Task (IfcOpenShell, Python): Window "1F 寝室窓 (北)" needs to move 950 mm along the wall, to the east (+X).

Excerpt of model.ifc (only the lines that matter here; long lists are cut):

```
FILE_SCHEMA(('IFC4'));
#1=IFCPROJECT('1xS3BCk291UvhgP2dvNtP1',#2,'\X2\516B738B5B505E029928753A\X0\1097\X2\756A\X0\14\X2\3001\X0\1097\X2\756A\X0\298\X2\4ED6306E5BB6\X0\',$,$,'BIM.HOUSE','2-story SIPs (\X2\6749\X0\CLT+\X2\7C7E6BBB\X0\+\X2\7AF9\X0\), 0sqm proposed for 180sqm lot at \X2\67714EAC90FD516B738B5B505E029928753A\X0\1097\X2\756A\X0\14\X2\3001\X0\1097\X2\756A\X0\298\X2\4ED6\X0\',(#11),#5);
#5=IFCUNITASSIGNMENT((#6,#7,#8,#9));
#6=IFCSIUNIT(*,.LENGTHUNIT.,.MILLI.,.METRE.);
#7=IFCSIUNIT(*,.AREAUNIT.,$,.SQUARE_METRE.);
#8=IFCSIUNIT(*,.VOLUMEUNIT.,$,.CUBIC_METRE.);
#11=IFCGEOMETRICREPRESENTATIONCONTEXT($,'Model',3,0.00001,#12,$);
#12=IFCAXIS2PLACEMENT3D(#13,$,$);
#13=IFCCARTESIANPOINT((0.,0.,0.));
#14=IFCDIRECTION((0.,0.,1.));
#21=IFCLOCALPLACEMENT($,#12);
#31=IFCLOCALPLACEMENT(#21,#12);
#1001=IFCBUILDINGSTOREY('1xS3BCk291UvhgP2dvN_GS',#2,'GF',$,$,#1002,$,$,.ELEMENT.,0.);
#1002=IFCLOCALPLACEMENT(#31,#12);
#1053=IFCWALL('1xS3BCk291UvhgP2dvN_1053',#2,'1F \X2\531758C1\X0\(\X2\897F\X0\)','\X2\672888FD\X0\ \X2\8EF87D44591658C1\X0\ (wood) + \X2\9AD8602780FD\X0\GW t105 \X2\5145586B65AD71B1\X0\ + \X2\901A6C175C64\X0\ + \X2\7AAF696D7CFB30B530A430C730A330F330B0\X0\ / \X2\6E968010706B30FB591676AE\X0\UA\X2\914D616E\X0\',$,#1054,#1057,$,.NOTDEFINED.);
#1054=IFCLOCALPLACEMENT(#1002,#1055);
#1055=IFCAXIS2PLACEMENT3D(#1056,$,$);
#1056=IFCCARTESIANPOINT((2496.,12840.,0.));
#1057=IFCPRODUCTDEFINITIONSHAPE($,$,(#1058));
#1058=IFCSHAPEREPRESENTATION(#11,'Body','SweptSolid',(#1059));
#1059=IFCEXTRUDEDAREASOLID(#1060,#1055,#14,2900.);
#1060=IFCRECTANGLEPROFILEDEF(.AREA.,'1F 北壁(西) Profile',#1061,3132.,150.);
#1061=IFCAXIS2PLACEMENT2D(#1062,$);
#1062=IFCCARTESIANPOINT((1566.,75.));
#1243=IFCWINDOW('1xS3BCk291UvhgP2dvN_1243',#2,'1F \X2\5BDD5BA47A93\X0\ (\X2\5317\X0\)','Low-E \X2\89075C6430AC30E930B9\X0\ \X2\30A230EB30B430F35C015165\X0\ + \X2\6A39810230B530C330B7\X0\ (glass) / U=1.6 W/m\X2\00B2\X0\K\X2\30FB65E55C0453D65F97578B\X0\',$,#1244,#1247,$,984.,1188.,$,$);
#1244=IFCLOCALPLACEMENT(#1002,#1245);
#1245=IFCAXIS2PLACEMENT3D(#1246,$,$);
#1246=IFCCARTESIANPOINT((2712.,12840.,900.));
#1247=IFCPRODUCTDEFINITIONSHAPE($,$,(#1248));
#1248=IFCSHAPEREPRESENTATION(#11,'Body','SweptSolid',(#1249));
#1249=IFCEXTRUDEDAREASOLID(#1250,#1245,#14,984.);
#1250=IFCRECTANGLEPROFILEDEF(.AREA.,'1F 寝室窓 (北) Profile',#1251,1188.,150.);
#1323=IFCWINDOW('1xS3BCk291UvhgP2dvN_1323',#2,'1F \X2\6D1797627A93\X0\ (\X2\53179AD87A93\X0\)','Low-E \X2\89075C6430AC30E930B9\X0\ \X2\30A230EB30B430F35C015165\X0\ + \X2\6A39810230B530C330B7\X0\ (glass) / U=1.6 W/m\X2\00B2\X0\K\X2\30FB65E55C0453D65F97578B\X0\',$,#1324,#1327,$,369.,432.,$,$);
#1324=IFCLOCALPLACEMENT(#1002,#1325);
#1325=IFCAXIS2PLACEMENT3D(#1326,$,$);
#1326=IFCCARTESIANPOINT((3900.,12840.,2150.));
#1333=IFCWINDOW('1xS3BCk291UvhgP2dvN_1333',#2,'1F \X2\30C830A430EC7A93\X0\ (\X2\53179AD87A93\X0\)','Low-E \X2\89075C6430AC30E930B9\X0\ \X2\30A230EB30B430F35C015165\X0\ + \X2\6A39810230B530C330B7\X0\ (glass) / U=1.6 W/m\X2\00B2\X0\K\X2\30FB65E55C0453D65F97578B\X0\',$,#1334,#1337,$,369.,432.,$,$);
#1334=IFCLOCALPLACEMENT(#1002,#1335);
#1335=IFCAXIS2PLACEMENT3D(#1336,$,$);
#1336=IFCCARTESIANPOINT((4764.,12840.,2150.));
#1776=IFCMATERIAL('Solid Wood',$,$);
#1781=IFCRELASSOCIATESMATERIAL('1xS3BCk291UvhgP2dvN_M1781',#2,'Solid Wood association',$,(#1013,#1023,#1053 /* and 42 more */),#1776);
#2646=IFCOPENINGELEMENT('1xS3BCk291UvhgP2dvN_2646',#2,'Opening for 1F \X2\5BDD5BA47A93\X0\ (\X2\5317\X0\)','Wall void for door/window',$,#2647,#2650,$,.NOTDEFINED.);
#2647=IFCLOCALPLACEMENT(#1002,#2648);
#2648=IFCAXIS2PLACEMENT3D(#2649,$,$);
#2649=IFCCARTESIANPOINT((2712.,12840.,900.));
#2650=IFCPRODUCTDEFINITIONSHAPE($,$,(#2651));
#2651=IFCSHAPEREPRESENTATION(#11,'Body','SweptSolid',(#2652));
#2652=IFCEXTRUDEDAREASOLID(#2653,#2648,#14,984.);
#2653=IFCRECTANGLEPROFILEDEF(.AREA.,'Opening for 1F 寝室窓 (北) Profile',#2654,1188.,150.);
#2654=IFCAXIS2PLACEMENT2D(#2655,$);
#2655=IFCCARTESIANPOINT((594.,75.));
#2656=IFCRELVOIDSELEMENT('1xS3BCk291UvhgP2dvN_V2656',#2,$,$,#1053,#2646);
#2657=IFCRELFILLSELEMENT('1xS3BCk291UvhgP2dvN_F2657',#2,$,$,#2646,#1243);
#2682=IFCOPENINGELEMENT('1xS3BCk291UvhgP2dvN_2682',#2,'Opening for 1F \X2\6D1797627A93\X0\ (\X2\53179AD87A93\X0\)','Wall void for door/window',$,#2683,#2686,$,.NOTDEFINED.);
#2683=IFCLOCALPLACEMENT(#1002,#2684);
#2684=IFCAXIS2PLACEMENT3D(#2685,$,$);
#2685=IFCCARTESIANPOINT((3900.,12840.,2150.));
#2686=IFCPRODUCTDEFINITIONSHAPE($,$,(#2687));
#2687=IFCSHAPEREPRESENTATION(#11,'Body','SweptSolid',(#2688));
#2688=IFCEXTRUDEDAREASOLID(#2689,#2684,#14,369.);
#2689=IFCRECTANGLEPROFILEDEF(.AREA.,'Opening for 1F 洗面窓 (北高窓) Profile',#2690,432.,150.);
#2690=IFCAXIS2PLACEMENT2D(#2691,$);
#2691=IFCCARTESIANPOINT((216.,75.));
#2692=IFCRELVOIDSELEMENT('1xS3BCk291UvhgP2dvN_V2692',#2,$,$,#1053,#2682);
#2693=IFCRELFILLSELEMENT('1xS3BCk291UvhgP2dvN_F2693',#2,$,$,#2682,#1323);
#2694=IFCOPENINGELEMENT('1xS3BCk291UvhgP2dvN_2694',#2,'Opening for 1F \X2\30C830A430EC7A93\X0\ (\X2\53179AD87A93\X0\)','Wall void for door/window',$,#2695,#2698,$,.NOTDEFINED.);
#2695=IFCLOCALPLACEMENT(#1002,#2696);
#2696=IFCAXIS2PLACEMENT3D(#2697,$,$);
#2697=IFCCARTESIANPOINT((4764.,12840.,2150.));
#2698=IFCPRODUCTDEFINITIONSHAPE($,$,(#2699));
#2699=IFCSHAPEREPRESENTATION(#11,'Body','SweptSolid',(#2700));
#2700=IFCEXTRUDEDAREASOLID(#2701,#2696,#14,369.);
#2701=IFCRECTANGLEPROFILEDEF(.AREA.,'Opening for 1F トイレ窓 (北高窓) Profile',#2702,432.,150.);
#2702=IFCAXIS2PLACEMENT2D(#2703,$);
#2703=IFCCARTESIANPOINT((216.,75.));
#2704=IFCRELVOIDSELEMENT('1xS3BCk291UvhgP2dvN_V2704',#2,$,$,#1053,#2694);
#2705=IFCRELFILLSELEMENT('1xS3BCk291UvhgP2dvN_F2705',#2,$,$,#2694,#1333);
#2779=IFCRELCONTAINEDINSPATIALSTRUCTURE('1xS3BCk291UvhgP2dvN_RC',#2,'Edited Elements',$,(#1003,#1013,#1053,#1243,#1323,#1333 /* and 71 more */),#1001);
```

```python
import ifcopenshell
import ifcopenshell.api.geometry
import ifcopenshell.util.placement
import ifcopenshell.util.unit

model = ifcopenshell.open("model.ifc")
unit_scale = ifcopenshell.util.unit.calculate_unit_scale(model)

window = model.by_id(1243)
opening = window.FillsVoids[0].RelatingOpeningElement
wall = opening.VoidsElements[0].RelatingBuildingElement

wall_matrix = ifcopenshell.util.placement.get_local_placement(wall.ObjectPlacement)
shift = wall_matrix[:3, 0] * 0.95 / unit_scale
before = ifcopenshell.util.placement.get_local_placement(window.ObjectPlacement)[:3, 3].copy()

# The window is not placed relative to its opening, so move both.
for product in (opening, window):
    matrix = ifcopenshell.util.placement.get_local_placement(product.ObjectPlacement)
    matrix[:3, 3] += shift
    ifcopenshell.api.geometry.edit_object_placement(model, product=product, matrix=matrix, is_si=False)

after = ifcopenshell.util.placement.get_local_placement(window.ObjectPlacement)[:3, 3]
print("window moved by", (after - before).round(3) + 0.0)

model.write("model-out.ifc")
```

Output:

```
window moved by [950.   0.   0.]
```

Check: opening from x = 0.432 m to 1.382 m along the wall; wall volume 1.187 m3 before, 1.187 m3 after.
